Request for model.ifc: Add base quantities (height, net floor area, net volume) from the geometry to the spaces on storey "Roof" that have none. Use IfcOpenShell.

First a look at what the model holds.

```python
import ifcopenshell
import ifcopenshell.util.element
import ifcopenshell.util.unit

model = ifcopenshell.open("model.ifc")
print(model.schema)
for unit_type in ("LENGTHUNIT", "AREAUNIT", "VOLUMEUNIT"):
    print(unit_type, ifcopenshell.util.unit.calculate_unit_scale(model, unit_type))
storey = next(s for s in model.by_type("IfcBuildingStorey") if s.Name == "Roof")
spaces = [e for e in ifcopenshell.util.element.get_decomposition(storey) if e.is_a("IfcSpace")]
for e in sorted(spaces, key=lambda e: e.id()):
    print(e.id(), e.is_a(), e.Name, list(ifcopenshell.util.element.get_psets(e, qtos_only=True)), sep=" | ")
```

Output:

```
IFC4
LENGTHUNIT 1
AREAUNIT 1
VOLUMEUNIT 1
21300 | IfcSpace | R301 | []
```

```python
import ifcopenshell
import ifcopenshell.api.pset
import ifcopenshell.geom
import ifcopenshell.util.element
import ifcopenshell.util.shape
import ifcopenshell.util.unit

model = ifcopenshell.open("model.ifc")
unit_scale = ifcopenshell.util.unit.calculate_unit_scale(model)
area_scale = ifcopenshell.util.unit.calculate_unit_scale(model, "AREAUNIT")
volume_scale = ifcopenshell.util.unit.calculate_unit_scale(model, "VOLUMEUNIT")
settings = ifcopenshell.geom.settings()

storey = next(s for s in model.by_type("IfcBuildingStorey") if s.Name == "Roof")
spaces = [e for e in ifcopenshell.util.element.get_decomposition(storey) if e.is_a("IfcSpace")]

for e in sorted(spaces, key=lambda e: e.id()):
    if ifcopenshell.util.element.get_psets(e, qtos_only=True, should_inherit=False):
        continue
    # Geometry comes back in metres, in the element's own axes.
    shape = ifcopenshell.geom.create_shape(settings, e)
    values = {
        "Height": ifcopenshell.util.shape.get_z(shape.geometry) / unit_scale,
        "NetFloorArea": ifcopenshell.util.shape.get_footprint_area(shape.geometry) / area_scale,
        "NetVolume": ifcopenshell.util.shape.get_volume(shape.geometry) / volume_scale,
    }
    qto = ifcopenshell.api.pset.add_qto(model, product=e, name="Qto_SpaceBaseQuantities")
    ifcopenshell.api.pset.edit_qto(model, qto=qto, properties=values)
    print(e.id(), {k: round(v, 3) for k, v in values.items()})

model.write("model_edited.ifc")
```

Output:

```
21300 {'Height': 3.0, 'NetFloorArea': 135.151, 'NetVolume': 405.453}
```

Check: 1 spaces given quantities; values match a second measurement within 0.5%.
